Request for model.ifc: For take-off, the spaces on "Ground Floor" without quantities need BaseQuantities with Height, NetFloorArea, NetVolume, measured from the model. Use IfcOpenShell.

First a look at what the model holds.

```python
import ifcopenshell
import ifcopenshell.util.element
import ifcopenshell.util.unit

model = ifcopenshell.open("model.ifc")
print(model.schema)
for unit_type in ("LENGTHUNIT", "AREAUNIT", "VOLUMEUNIT"):
    print(unit_type, ifcopenshell.util.unit.calculate_unit_scale(model, unit_type))
storey = next(s for s in model.by_type("IfcBuildingStorey") if s.Name == "Ground Floor")
spaces = [e for e in ifcopenshell.util.element.get_decomposition(storey) if e.is_a("IfcSpace")]
for e in sorted(spaces, key=lambda e: e.id()):
    print(e.id(), e.is_a(), e.Name, list(ifcopenshell.util.element.get_psets(e, qtos_only=True)), sep=" | ")
```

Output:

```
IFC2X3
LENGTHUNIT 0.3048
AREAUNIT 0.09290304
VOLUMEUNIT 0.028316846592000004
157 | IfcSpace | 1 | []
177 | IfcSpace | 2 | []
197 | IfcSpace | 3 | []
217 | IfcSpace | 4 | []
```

```python
import ifcopenshell
import ifcopenshell.api.pset
import ifcopenshell.geom
import ifcopenshell.util.element
import ifcopenshell.util.shape
import ifcopenshell.util.unit

model = ifcopenshell.open("model.ifc")
unit_scale = ifcopenshell.util.unit.calculate_unit_scale(model)
area_scale = ifcopenshell.util.unit.calculate_unit_scale(model, "AREAUNIT")
volume_scale = ifcopenshell.util.unit.calculate_unit_scale(model, "VOLUMEUNIT")
settings = ifcopenshell.geom.settings()

storey = next(s for s in model.by_type("IfcBuildingStorey") if s.Name == "Ground Floor")
spaces = [e for e in ifcopenshell.util.element.get_decomposition(storey) if e.is_a("IfcSpace")]

for e in sorted(spaces, key=lambda e: e.id()):
    if ifcopenshell.util.element.get_psets(e, qtos_only=True, should_inherit=False):
        continue
    # Geometry comes back in metres, in the element's own axes.
    shape = ifcopenshell.geom.create_shape(settings, e)
    values = {
        "Height": ifcopenshell.util.shape.get_z(shape.geometry) / unit_scale,
        "NetFloorArea": ifcopenshell.util.shape.get_footprint_area(shape.geometry) / area_scale,
        "NetVolume": ifcopenshell.util.shape.get_volume(shape.geometry) / volume_scale,
    }
    qto = ifcopenshell.api.pset.add_qto(model, product=e, name="BaseQuantities")
    ifcopenshell.api.pset.edit_qto(model, qto=qto, properties=values)
    print(e.id(), {k: round(v, 3) for k, v in values.items()})

model.write("model_v2.ifc")
```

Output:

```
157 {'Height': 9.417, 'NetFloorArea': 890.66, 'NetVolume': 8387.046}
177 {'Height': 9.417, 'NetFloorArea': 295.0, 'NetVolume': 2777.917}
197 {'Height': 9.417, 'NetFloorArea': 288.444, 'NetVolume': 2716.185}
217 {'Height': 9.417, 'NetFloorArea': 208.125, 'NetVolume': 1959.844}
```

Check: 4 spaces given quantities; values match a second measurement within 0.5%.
